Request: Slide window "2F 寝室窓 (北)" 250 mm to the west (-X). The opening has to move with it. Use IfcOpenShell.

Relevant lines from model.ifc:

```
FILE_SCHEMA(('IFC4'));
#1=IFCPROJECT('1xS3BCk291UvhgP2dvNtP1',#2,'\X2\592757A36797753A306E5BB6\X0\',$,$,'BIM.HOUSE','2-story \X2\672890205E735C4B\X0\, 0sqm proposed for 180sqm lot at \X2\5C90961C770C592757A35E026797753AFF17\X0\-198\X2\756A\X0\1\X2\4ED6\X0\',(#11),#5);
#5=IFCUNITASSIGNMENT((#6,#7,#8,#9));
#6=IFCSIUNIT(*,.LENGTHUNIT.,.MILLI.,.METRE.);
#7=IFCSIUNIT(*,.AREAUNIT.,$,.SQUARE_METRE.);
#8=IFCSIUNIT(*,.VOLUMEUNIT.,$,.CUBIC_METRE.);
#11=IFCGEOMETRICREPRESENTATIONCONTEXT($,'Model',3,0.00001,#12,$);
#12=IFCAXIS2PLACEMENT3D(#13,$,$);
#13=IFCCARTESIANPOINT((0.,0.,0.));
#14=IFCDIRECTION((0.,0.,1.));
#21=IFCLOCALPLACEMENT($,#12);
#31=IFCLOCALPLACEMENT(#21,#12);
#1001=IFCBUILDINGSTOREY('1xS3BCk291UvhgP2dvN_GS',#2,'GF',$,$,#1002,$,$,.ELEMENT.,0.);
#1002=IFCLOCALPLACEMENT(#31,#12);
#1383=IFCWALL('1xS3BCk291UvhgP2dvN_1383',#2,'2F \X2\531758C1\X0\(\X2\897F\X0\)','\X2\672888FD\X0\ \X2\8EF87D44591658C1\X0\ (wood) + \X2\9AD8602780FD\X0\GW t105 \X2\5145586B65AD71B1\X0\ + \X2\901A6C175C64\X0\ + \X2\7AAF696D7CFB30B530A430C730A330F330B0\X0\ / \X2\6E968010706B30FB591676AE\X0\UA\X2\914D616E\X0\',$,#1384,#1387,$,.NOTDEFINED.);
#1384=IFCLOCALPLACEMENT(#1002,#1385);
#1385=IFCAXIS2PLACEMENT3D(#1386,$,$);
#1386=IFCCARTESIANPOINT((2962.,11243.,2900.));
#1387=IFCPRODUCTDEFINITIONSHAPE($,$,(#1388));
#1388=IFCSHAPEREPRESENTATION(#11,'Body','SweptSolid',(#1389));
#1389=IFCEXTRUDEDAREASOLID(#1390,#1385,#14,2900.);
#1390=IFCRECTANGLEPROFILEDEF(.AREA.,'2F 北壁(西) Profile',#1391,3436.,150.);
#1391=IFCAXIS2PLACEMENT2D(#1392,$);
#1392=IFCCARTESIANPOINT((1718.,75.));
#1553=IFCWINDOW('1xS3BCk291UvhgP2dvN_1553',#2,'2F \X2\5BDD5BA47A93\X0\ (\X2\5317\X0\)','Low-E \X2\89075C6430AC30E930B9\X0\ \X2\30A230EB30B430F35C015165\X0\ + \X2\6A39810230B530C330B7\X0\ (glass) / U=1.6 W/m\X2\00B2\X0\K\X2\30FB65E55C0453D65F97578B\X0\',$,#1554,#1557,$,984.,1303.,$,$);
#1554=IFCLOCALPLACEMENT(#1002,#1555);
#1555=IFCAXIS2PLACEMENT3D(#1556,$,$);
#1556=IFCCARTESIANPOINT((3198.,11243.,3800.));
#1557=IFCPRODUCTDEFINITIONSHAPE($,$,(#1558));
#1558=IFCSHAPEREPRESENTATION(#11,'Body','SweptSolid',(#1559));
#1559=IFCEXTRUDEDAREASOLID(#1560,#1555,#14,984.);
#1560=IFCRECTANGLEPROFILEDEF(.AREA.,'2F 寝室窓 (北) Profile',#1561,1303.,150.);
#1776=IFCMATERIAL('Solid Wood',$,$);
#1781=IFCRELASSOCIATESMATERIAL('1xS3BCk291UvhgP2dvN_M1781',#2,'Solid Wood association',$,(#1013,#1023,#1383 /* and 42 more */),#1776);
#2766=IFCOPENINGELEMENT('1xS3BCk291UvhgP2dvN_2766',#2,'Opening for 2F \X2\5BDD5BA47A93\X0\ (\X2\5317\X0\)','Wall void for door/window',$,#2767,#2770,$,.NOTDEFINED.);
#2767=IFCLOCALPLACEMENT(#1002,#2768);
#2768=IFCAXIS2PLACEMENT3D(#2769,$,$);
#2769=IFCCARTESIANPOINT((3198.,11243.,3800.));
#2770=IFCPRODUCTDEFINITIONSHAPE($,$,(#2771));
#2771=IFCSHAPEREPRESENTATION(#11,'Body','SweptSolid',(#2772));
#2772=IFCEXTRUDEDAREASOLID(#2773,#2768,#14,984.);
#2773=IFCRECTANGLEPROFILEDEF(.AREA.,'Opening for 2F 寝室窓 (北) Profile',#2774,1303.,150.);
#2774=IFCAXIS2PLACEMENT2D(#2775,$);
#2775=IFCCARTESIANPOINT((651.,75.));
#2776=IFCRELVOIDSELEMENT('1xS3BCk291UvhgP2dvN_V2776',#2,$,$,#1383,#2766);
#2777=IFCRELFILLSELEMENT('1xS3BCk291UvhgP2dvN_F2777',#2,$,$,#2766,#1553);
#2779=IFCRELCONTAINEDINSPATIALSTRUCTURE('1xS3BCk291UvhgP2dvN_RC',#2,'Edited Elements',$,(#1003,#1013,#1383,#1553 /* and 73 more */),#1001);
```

```python
import ifcopenshell
import ifcopenshell.api.geometry
import ifcopenshell.util.placement
import ifcopenshell.util.unit

model = ifcopenshell.open("model.ifc")
unit_scale = ifcopenshell.util.unit.calculate_unit_scale(model)

window = model.by_id(1553)
opening = window.FillsVoids[0].RelatingOpeningElement
wall = opening.VoidsElements[0].RelatingBuildingElement

wall_matrix = ifcopenshell.util.placement.get_local_placement(wall.ObjectPlacement)
shift = wall_matrix[:3, 0] * -0.25 / unit_scale
before = ifcopenshell.util.placement.get_local_placement(window.ObjectPlacement)[:3, 3].copy()

# The window is not placed relative to its opening, so move both.
for product in (opening, window):
    matrix = ifcopenshell.util.placement.get_local_placement(product.ObjectPlacement)
    matrix[:3, 3] += shift
    ifcopenshell.api.geometry.edit_object_placement(model, product=product, matrix=matrix, is_si=False)

after = ifcopenshell.util.placement.get_local_placement(window.ObjectPlacement)[:3, 3]
print("window moved by", (after - before).round(3) + 0.0)

model.write("model_v2.ifc")
```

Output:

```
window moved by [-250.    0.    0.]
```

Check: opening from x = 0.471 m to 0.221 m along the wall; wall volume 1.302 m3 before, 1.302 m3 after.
